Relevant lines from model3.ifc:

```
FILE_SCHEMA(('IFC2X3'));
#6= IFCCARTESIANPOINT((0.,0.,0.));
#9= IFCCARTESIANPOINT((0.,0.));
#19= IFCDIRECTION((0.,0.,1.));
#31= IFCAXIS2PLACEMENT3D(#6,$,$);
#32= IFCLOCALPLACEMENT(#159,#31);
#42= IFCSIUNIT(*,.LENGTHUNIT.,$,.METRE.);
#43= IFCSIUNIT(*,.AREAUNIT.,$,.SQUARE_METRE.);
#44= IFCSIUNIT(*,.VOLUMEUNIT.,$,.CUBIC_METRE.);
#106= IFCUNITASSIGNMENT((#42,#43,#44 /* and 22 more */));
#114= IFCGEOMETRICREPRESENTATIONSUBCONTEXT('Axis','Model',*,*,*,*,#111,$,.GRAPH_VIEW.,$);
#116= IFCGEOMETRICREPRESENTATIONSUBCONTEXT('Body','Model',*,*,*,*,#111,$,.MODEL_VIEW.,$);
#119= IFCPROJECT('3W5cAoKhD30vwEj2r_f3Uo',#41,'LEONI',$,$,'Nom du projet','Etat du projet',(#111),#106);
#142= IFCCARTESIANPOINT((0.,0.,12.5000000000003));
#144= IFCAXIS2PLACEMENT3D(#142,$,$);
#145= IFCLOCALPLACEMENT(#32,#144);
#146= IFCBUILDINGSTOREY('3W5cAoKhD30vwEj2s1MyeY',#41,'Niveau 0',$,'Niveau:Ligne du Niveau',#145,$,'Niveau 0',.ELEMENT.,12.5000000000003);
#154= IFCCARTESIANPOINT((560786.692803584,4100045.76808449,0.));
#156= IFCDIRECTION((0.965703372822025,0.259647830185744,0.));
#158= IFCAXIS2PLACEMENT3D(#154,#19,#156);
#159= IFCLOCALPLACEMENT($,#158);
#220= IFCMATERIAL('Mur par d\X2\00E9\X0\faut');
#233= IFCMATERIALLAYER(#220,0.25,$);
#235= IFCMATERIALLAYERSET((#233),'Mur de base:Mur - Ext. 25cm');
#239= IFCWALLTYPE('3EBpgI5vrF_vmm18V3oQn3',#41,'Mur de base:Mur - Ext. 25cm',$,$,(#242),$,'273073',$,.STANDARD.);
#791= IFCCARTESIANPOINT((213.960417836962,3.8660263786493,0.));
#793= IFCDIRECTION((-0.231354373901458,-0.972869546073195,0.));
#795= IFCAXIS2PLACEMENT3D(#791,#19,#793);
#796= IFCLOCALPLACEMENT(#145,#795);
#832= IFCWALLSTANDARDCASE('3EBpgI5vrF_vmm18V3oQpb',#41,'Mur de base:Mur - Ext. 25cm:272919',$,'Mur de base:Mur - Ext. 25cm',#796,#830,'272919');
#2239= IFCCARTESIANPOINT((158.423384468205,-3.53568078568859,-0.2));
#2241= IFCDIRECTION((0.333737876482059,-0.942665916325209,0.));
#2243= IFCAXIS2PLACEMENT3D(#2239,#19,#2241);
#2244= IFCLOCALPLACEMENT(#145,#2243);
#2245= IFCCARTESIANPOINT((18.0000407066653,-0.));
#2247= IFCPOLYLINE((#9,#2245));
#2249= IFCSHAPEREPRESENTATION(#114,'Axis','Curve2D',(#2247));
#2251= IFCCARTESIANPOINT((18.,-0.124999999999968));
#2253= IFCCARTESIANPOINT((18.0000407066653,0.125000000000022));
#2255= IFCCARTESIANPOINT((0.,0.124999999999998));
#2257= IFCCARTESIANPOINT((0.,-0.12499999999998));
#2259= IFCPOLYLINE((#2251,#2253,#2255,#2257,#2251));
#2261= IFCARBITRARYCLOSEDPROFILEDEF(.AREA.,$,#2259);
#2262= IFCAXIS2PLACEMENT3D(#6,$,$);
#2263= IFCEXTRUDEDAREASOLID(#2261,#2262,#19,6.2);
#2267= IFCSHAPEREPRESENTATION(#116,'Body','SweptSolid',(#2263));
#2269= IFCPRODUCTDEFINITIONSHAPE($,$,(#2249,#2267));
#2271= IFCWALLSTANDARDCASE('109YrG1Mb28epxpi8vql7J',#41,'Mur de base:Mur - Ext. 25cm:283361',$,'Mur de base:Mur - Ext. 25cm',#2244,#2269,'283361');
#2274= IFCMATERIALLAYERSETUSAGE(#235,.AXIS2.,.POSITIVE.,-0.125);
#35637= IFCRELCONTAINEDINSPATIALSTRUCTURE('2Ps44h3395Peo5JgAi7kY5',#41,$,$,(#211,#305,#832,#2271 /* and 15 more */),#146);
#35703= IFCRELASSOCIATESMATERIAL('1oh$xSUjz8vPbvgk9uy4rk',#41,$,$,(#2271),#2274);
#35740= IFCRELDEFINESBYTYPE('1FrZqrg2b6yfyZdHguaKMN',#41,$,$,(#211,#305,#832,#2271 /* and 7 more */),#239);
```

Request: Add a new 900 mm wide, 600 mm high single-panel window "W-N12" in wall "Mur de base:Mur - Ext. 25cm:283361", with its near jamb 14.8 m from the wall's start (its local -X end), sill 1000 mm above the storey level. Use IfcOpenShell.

```python
import numpy as np
import ifcopenshell
import ifcopenshell.api.feature
import ifcopenshell.api.geometry
import ifcopenshell.api.root
import ifcopenshell.api.spatial
import ifcopenshell.api.type
import ifcopenshell.geom
import ifcopenshell.util.element
import ifcopenshell.util.placement
import ifcopenshell.util.representation
import ifcopenshell.util.shape
import ifcopenshell.util.unit

model = ifcopenshell.open("model3.ifc")
unit_scale = ifcopenshell.util.unit.calculate_unit_scale(model)
settings = ifcopenshell.geom.settings()


def volume(element):
    """Net volume in cubic metres, openings subtracted."""
    shape = ifcopenshell.geom.create_shape(settings, element)
    return ifcopenshell.util.shape.get_volume(shape.geometry)


wall = model.by_guid("109YrG1Mb28epxpi8vql7J")
storey = ifcopenshell.util.element.get_container(wall, ifc_class="IfcBuildingStorey")
context = ifcopenshell.util.representation.get_context(model, "Model", "Body", "MODEL_VIEW")
before = volume(wall)

width, height, from_end, sill = 0.9, 0.6, 14.8, 1  # metres

# The wall runs along its own X axis, and the end named is its -X end.
wall_shape = ifcopenshell.geom.create_shape(settings, wall)
x, y, z = ifcopenshell.util.shape.get_vertices(wall_shape.geometry).T
start = x.min() + from_end
face, thickness = float(y.min()), float(y.max() - y.min())
wall_matrix = ifcopenshell.util.placement.get_local_placement(wall.ObjectPlacement)
level = ifcopenshell.util.placement.get_local_placement(storey.ObjectPlacement)[2, 3]


def in_wall(x, y):
    """Placement at x, y metres in the wall's axes, at sill height."""
    matrix = wall_matrix.copy()
    matrix[:, 3] = wall_matrix @ np.array([x / unit_scale, y / unit_scale, 0.0, 1.0])
    matrix[2, 3] = level + sill / unit_scale
    return matrix


# Opening: a box that overshoots both wall faces by 50 mm.
opening = ifcopenshell.api.root.create_entity(model, ifc_class="IfcOpeningElement")
box = ifcopenshell.api.geometry.add_wall_representation(
    model, context=context, length=width, height=height, thickness=thickness + 0.1
)
ifcopenshell.api.geometry.assign_representation(model, product=opening, representation=box)
ifcopenshell.api.geometry.edit_object_placement(model, product=opening, matrix=in_wall(start, face - 0.05), is_si=False)
ifcopenshell.api.feature.add_feature(model, feature=opening, element=wall)

window = ifcopenshell.api.root.create_entity(model, ifc_class="IfcWindow", name="W-N12")
window.OverallWidth, window.OverallHeight = width / unit_scale, height / unit_scale
body = ifcopenshell.api.geometry.add_window_representation(
    model,
    context=context,
    overall_width=window.OverallWidth,
    overall_height=window.OverallHeight,
    partition_type="SINGLE_PANEL",
)
ifcopenshell.api.geometry.assign_representation(model, product=window, representation=body)
ifcopenshell.api.spatial.assign_container(model, products=[window], relating_structure=storey)
fills = ifcopenshell.api.feature.add_filling(model, opening=opening, element=window)
fills.OwnerHistory = window.OwnerHistory  # required in IFC2X3

# IFC2X3 keeps the operation on the window style.
style = ifcopenshell.api.root.create_entity(model, ifc_class="IfcWindowStyle", name="W-N12")
style.OperationType, style.ConstructionType = "SINGLE_PANEL", "NOTDEFINED"
style.ParameterTakesPrecedence = style.Sizeable = False
ifcopenshell.api.type.assign_type(model, related_objects=[window], relating_type=style)

# Centre the window in the wall's thickness.
ifcopenshell.api.geometry.edit_object_placement(model, product=window, matrix=in_wall(start, face), is_si=False)
window_shape = ifcopenshell.geom.create_shape(settings, window)
depth = ifcopenshell.util.shape.get_vertices(window_shape.geometry)[:, 1]
offset = face + thickness / 2 - (depth.min() + depth.max()) / 2
ifcopenshell.api.geometry.edit_object_placement(model, product=window, matrix=in_wall(start, offset), is_si=False)

after = volume(wall)

print(f"wall volume {before:.3f} -> {after:.3f} m3")

model.write("model3_edited.ifc")
```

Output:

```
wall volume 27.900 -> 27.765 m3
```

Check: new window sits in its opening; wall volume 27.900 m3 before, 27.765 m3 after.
